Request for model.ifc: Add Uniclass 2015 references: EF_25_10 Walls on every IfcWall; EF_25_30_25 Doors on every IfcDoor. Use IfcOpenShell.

First a look at what the model holds.

```python
import ifcopenshell

model = ifcopenshell.open("model.ifc")
print(model.schema)
print("classifications:", [c.Name for c in model.by_type("IfcClassification")])
for ifc_class in ("IfcDoor", "IfcRoof", "IfcStair", "IfcWall", "IfcWindow"):
    print(ifc_class, len(model.by_type(ifc_class)))
```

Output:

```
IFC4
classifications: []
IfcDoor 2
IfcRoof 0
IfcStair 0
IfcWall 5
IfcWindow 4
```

```python
import ifcopenshell
import ifcopenshell.api.classification

model = ifcopenshell.open("model.ifc")

system = ifcopenshell.api.classification.add_classification(model, classification="Uniclass 2015")

codes = {
    "IfcWall": ("EF_25_10", "Walls"),
    "IfcDoor": ("EF_25_30_25", "Doors"),
}
for ifc_class, (code, name) in codes.items():
    products = model.by_type(ifc_class)
    ifcopenshell.api.classification.add_reference(
        model, products=products, classification=system, identification=code, name=name
    )
    print(code, len(products))

model.write("model-out.ifc")
```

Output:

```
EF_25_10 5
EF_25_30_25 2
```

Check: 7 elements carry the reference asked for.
